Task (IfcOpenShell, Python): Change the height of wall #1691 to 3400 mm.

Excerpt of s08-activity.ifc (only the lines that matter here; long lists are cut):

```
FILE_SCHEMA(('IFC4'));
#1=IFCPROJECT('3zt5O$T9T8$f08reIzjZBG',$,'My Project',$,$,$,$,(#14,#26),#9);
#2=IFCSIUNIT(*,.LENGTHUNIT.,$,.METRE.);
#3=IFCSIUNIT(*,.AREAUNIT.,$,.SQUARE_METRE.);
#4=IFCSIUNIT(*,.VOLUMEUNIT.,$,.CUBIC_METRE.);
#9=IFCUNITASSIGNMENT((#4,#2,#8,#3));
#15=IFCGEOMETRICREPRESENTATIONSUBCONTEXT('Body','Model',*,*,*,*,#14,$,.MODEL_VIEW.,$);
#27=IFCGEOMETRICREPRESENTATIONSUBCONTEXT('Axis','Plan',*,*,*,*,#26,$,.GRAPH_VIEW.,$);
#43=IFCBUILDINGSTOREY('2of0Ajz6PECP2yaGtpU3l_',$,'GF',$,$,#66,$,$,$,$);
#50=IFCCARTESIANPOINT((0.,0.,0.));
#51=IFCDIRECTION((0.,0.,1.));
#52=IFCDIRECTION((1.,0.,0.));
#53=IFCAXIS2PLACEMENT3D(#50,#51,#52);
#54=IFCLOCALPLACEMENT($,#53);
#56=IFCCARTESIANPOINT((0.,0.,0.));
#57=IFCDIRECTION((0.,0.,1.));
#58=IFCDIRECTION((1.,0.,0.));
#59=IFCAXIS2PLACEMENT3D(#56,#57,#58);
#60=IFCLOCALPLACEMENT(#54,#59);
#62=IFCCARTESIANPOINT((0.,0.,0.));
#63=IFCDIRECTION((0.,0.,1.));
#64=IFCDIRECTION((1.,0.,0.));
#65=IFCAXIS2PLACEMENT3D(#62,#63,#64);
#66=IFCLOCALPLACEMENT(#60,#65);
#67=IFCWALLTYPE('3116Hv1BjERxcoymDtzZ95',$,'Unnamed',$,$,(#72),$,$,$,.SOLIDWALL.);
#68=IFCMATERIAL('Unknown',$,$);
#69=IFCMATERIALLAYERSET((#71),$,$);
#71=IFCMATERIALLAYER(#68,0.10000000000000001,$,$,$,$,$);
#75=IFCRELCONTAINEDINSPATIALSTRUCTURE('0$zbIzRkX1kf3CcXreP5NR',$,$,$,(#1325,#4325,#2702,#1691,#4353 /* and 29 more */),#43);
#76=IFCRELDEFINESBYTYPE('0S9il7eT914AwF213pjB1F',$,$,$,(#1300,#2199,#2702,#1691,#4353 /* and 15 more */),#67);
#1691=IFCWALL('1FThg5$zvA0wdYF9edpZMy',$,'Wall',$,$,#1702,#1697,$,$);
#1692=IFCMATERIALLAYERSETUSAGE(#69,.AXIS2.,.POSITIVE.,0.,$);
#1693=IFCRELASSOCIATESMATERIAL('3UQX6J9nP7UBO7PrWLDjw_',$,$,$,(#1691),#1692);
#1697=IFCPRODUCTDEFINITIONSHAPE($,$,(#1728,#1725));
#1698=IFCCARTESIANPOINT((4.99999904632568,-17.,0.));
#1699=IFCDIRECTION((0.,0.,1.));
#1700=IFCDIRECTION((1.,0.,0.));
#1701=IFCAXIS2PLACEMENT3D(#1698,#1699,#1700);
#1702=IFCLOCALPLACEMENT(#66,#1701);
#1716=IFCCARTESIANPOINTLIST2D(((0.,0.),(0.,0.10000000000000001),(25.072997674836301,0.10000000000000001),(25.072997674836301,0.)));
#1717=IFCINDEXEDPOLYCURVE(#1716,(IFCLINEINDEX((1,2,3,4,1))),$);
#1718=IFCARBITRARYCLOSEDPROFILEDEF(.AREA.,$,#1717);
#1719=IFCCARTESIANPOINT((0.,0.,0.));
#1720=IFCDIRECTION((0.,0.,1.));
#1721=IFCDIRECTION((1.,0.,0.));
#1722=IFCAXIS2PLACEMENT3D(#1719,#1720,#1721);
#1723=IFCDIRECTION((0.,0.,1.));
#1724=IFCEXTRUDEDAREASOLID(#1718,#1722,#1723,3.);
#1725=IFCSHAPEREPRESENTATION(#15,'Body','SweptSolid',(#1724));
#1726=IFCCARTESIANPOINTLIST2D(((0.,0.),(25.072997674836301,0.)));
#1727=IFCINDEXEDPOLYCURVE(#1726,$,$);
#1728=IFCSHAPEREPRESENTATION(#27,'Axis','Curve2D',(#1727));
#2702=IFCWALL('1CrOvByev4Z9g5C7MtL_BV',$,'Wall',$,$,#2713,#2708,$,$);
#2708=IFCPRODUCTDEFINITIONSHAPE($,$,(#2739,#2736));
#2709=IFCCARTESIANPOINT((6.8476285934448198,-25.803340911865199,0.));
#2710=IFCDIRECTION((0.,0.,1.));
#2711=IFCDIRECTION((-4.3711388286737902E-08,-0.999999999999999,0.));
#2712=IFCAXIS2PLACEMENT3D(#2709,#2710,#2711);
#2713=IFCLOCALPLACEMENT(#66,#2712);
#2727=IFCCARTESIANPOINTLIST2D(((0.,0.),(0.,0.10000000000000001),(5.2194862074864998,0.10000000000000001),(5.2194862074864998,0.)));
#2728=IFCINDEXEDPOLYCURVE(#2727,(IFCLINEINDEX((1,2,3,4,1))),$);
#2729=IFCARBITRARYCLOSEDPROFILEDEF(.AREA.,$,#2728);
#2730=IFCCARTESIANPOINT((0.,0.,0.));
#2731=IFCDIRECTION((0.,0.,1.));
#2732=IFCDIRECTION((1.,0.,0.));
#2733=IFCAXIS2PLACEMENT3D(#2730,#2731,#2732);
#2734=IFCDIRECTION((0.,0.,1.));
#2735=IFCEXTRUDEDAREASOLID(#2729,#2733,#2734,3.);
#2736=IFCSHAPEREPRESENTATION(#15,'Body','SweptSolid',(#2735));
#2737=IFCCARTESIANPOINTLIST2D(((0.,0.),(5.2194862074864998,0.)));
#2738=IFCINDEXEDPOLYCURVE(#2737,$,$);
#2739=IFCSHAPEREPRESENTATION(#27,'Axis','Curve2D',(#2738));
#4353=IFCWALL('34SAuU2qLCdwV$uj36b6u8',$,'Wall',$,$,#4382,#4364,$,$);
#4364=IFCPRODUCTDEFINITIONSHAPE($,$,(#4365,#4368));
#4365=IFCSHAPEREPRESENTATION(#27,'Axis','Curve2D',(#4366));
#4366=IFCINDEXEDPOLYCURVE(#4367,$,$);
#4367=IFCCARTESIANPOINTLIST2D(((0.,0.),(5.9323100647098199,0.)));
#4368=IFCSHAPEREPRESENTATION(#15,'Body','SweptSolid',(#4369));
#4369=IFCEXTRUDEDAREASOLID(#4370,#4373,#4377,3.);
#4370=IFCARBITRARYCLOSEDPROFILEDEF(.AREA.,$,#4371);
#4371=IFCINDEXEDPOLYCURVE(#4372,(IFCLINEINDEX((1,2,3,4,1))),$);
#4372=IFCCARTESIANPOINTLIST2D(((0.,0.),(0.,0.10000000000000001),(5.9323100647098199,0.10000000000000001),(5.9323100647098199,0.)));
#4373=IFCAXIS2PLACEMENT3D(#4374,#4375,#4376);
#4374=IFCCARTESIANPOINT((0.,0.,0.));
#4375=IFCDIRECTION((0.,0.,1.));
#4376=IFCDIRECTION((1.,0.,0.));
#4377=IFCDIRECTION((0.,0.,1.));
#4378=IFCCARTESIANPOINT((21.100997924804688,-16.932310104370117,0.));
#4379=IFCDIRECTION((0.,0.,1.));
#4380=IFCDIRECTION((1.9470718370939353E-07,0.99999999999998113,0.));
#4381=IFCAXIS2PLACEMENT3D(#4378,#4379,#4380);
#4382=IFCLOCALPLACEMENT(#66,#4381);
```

```python
import ifcopenshell
import ifcopenshell.geom
import ifcopenshell.util.representation
import ifcopenshell.util.shape

model = ifcopenshell.open("s08-activity.ifc")
settings = ifcopenshell.geom.settings()


def volume(element):
    """Net volume in cubic metres, openings subtracted."""
    shape = ifcopenshell.geom.create_shape(settings, element)
    return ifcopenshell.util.shape.get_volume(shape.geometry)


wall = model.by_guid("1FThg5$zvA0wdYF9edpZMy")
before = volume(wall)

body = ifcopenshell.util.representation.get_representation(wall, "Model", "Body")
solid = body.Items[0]
old_height = solid.Depth
solid.Depth = 3.4
after = volume(wall)

print(f"height {old_height:g} -> {solid.Depth:g}, volume {before:.3f} -> {after:.3f} m3")

model.write("s08-activity_rev.ifc")
```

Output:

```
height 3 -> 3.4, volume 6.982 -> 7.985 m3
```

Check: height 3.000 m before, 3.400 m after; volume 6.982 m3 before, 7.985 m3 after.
